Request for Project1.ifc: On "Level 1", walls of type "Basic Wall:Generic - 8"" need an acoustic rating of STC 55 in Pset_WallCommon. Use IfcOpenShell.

First a look at what the model holds.

```python
import ifcopenshell
import ifcopenshell.util.element

model = ifcopenshell.open("Project1.ifc")
print(model.schema)
storey = next(s for s in model.by_type("IfcBuildingStorey") if s.Name == "Level 1")
walls = [e for e in ifcopenshell.util.element.get_decomposition(storey) if e.is_a("IfcWall")]
seen = {}
for e in walls:
    element_type = ifcopenshell.util.element.get_type(e)
    key = (element_type.Name if element_type != e and element_type else None, ifcopenshell.util.element.get_pset(e, "Pset_WallCommon", "AcousticRating"))
    seen[key] = seen.get(key, 0) + 1
for (name, value), count in sorted(seen.items(), key=str):
    print(count, "x", name, "|", value)
```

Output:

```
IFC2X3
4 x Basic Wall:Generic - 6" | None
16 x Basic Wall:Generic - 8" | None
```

```python
import ifcopenshell
import ifcopenshell.api.pset
import ifcopenshell.util.element

model = ifcopenshell.open("Project1.ifc")

storey = next(s for s in model.by_type("IfcBuildingStorey") if s.Name == "Level 1")
walls = [e for e in ifcopenshell.util.element.get_decomposition(storey) if e.is_a("IfcWall")]

count = 0
for e in walls:
    element_type = ifcopenshell.util.element.get_type(e)
    if element_type in (None, e) or element_type.Name != 'Basic Wall:Generic - 8"':
        continue
    # add_pset returns the element's existing set when there is one.
    pset = ifcopenshell.api.pset.add_pset(model, product=e, name="Pset_WallCommon")
    ifcopenshell.api.pset.edit_pset(model, pset=pset, properties={"AcousticRating": "STC 55"})
    count += 1

print(count, "walls updated")

model.write("Project1_v2.ifc")
```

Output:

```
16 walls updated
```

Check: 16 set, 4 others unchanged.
